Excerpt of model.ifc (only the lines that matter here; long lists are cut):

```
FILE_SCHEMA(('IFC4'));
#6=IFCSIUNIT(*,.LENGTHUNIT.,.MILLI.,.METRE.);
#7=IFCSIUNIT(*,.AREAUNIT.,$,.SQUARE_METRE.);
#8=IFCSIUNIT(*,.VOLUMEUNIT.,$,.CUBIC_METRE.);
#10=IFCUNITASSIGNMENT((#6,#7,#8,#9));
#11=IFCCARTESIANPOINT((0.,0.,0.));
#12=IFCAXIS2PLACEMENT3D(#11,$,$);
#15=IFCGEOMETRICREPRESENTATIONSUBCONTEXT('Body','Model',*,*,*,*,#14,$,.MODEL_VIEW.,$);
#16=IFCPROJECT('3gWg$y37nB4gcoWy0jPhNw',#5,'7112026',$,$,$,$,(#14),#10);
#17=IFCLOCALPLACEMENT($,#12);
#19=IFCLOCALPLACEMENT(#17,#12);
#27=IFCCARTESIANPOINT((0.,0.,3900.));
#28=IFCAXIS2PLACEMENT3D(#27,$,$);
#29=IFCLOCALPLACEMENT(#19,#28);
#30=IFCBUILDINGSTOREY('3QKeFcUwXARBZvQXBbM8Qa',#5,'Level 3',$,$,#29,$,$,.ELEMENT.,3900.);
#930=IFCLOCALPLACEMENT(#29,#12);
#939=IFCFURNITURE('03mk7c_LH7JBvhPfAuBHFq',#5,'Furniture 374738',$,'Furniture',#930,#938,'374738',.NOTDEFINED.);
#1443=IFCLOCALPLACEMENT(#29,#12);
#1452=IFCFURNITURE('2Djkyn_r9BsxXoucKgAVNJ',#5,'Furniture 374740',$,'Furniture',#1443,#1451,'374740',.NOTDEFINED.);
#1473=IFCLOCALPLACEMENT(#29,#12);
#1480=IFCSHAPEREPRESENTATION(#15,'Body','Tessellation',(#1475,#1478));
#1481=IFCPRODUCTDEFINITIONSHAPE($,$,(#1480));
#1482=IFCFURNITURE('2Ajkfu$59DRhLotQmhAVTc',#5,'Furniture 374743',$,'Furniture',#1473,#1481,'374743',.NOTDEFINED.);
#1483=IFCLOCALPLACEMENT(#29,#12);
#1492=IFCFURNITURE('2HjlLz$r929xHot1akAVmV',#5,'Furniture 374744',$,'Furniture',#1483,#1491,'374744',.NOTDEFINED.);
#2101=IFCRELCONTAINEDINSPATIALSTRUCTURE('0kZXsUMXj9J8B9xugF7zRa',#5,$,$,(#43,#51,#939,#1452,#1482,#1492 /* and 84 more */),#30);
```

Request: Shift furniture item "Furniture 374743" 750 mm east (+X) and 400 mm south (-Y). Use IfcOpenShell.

```python
import ifcopenshell
import ifcopenshell.api.geometry
import ifcopenshell.util.placement

model = ifcopenshell.open("model.ifc")

item = model.by_guid("2Ajkfu$59DRhLotQmhAVTc")
matrix = ifcopenshell.util.placement.get_local_placement(item.ObjectPlacement)
matrix[0, 3] += 750.0
matrix[1, 3] -= 400.0
ifcopenshell.api.geometry.edit_object_placement(model, product=item, matrix=matrix, is_si=False)

print(ifcopenshell.util.placement.get_local_placement(item.ObjectPlacement).round(3) + 0.0)

model.write("model_edited.ifc")
```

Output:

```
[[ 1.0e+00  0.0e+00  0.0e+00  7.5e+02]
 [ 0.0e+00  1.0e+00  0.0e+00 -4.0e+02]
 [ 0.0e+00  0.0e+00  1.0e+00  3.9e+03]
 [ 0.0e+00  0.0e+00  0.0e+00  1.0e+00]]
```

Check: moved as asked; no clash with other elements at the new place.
